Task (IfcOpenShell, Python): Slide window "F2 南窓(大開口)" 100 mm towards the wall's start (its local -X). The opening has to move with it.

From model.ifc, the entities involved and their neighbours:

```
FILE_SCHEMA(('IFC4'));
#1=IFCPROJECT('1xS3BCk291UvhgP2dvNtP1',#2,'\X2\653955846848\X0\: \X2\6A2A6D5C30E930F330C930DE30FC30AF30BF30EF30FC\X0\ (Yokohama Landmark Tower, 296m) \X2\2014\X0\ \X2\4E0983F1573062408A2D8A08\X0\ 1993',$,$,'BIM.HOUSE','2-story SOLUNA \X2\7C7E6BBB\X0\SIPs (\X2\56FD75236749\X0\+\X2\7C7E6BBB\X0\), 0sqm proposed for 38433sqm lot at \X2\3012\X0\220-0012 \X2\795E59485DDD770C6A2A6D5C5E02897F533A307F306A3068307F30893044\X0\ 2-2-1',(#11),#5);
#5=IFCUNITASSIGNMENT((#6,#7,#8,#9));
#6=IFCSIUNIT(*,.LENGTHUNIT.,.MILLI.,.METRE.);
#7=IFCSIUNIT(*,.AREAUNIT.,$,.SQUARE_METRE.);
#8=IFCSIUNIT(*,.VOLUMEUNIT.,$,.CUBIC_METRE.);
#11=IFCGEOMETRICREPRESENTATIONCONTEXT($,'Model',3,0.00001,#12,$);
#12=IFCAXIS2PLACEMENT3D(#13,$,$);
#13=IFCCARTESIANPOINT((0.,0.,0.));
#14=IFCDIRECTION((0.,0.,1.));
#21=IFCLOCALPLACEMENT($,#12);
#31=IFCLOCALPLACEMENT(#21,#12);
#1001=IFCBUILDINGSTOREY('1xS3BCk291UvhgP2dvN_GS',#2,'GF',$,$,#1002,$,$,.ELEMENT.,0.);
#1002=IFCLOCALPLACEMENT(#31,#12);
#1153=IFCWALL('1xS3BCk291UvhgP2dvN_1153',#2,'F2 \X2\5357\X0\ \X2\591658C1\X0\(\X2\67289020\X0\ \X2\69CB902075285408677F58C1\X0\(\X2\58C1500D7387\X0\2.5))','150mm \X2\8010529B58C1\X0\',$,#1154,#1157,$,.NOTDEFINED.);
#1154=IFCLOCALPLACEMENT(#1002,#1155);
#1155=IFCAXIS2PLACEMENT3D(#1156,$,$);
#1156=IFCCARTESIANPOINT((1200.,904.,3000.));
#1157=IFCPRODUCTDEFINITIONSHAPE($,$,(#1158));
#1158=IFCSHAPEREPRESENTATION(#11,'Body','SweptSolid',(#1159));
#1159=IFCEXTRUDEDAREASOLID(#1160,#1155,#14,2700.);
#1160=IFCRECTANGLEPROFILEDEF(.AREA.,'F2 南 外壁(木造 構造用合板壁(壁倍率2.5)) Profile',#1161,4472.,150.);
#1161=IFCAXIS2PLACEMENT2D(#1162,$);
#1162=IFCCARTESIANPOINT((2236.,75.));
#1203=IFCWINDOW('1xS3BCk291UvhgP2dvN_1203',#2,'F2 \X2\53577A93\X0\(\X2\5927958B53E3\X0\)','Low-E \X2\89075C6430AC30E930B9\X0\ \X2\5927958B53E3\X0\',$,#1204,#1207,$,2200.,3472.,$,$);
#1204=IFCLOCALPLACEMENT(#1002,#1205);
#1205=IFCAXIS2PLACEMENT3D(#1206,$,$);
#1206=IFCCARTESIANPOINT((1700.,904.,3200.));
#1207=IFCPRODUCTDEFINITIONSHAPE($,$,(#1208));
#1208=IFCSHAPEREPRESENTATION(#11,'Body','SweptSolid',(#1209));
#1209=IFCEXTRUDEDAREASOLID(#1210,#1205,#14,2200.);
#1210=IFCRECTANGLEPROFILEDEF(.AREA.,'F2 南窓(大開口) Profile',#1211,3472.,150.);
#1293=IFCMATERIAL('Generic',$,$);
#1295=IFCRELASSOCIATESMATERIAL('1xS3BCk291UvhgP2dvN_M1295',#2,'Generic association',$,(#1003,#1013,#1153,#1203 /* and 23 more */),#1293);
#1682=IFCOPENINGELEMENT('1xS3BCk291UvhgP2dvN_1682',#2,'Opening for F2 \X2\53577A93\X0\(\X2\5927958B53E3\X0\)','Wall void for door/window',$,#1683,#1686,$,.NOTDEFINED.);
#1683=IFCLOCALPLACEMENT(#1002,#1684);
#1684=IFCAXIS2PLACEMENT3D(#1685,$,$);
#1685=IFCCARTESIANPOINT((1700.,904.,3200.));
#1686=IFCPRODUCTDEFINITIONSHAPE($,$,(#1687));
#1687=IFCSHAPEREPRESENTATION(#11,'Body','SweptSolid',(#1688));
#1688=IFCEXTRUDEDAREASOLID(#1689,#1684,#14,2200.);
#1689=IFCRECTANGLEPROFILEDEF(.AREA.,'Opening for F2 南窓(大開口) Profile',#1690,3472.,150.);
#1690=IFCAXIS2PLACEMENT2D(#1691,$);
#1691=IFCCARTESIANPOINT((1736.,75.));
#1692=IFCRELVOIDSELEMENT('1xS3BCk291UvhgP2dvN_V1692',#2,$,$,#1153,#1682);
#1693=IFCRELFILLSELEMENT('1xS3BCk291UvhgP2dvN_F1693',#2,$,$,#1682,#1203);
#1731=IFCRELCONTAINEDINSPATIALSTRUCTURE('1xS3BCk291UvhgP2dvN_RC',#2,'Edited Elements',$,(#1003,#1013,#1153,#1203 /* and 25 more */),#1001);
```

```python
import ifcopenshell
import ifcopenshell.api.geometry
import ifcopenshell.util.placement

model = ifcopenshell.open("model.ifc")

window = model.by_guid("1xS3BCk291UvhgP2dvN_1203")
opening = window.FillsVoids[0].RelatingOpeningElement
wall = opening.VoidsElements[0].RelatingBuildingElement

wall_matrix = ifcopenshell.util.placement.get_local_placement(wall.ObjectPlacement)
shift = wall_matrix[:3, 0] * -100.0
before = ifcopenshell.util.placement.get_local_placement(window.ObjectPlacement)[:3, 3].copy()

# The window is not placed relative to its opening, so move both.
for product in (opening, window):
    matrix = ifcopenshell.util.placement.get_local_placement(product.ObjectPlacement)
    matrix[:3, 3] += shift
    ifcopenshell.api.geometry.edit_object_placement(model, product=product, matrix=matrix, is_si=False)

after = ifcopenshell.util.placement.get_local_placement(window.ObjectPlacement)[:3, 3]
print("window moved by", (after - before).round(3) + 0.0)

model.write("model_updated.ifc")
```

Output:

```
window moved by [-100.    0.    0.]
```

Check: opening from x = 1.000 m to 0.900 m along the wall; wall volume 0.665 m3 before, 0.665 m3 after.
